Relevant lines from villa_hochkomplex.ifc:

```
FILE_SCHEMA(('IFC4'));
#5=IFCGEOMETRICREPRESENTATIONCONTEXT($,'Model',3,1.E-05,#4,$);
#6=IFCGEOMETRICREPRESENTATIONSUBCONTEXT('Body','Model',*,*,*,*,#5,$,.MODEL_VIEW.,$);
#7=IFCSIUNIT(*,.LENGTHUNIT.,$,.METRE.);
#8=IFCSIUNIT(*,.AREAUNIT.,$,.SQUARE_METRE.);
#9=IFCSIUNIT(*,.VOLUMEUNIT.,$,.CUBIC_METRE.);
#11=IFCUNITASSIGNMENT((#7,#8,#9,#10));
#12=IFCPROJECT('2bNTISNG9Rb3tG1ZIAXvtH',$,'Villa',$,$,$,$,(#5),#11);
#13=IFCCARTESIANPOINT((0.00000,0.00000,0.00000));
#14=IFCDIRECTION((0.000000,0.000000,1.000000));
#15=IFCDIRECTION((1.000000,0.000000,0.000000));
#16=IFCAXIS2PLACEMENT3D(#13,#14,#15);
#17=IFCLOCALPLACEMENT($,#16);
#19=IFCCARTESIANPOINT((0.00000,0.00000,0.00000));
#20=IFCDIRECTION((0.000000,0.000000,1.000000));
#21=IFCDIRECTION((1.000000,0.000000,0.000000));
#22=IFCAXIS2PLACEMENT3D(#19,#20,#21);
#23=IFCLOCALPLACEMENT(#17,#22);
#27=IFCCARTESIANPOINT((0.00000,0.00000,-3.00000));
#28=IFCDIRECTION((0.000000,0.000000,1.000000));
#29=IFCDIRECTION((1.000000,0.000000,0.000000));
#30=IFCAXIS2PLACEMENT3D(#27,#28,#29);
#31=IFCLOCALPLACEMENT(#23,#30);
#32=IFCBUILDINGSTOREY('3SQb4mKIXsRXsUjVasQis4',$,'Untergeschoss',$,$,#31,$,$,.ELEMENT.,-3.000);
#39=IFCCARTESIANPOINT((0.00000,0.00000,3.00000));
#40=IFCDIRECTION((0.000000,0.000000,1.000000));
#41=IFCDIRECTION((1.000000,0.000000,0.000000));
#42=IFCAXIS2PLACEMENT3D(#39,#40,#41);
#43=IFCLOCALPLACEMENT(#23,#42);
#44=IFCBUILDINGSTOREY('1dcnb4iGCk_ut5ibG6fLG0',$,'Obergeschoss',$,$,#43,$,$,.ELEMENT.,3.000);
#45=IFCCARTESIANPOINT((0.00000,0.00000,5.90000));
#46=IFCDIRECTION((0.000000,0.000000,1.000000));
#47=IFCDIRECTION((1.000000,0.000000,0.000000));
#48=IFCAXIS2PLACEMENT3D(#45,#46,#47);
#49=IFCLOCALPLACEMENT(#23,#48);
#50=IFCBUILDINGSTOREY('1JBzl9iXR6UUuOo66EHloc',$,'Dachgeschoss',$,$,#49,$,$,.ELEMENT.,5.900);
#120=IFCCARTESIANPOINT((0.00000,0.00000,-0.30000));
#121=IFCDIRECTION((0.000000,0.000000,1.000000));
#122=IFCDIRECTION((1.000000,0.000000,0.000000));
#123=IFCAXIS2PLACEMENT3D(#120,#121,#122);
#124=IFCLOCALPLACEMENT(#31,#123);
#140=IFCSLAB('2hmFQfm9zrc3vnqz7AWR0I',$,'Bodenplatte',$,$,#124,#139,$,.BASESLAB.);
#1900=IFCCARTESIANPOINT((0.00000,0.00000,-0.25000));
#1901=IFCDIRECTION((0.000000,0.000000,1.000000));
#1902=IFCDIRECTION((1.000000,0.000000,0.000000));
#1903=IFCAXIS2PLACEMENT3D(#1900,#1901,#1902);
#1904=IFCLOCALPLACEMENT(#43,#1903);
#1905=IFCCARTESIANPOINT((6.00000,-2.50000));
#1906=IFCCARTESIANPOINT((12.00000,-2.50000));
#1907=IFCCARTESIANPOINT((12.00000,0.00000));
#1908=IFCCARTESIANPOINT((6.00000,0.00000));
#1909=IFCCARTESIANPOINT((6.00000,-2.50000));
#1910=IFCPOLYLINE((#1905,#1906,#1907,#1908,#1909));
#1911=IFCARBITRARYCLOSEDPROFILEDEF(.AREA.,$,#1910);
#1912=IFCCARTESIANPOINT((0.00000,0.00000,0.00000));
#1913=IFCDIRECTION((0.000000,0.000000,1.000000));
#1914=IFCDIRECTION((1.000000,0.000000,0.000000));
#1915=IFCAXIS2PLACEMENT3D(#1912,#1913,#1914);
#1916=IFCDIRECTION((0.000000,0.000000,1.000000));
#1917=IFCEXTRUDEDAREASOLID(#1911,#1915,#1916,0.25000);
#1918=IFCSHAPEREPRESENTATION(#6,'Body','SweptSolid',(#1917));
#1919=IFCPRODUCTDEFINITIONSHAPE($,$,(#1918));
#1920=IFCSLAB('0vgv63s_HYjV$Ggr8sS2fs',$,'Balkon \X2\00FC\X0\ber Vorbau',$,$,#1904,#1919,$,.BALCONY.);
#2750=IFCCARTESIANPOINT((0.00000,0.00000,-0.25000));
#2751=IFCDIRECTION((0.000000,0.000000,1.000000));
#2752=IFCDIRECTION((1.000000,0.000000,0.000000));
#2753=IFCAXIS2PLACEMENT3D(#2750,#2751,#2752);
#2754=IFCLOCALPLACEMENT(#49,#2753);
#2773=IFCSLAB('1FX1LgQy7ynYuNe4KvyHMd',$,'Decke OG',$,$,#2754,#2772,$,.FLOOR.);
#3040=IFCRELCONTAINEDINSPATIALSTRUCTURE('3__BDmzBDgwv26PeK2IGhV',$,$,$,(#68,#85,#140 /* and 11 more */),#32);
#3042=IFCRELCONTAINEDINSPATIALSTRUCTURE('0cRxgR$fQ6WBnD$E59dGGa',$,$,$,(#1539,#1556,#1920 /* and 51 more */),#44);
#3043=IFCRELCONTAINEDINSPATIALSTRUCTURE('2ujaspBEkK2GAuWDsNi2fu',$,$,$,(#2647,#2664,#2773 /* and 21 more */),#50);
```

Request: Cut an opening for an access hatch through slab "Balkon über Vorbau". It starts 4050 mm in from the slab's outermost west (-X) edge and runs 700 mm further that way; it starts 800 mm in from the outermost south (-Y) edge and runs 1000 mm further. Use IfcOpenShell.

```python
import numpy as np
import ifcopenshell
import ifcopenshell.api.feature
import ifcopenshell.api.geometry
import ifcopenshell.api.root
import ifcopenshell.geom
import ifcopenshell.util.placement
import ifcopenshell.util.representation
import ifcopenshell.util.shape
import ifcopenshell.util.unit

model = ifcopenshell.open("villa_hochkomplex.ifc")
unit_scale = ifcopenshell.util.unit.calculate_unit_scale(model)
settings = ifcopenshell.geom.settings()


def volume(element):
    """Net volume in cubic metres, openings subtracted."""
    shape = ifcopenshell.geom.create_shape(settings, element)
    return ifcopenshell.util.shape.get_volume(shape.geometry)


slab = model.by_guid("0vgv63s_HYjV$Ggr8sS2fs")
before = volume(slab)

# Extent in the slab's own axes, in metres. The edges named are its -X and -Y sides.
slab_shape = ifcopenshell.geom.create_shape(settings, slab)
vertices = ifcopenshell.util.shape.get_vertices(slab_shape.geometry)
x_min, y_min, bottom = vertices.min(axis=0)
top = vertices[:, 2].max()

opening = ifcopenshell.api.root.create_entity(model, ifc_class="IfcOpeningElement", name="Access hatch opening", predefined_type="OPENING")
context = ifcopenshell.util.representation.get_context(model, "Model", "Body", "MODEL_VIEW")
width, depth = 0.7, 1
outline = [(0.0, 0.0), (width, 0.0), (width, depth), (0.0, depth), (0.0, 0.0)]
# Overshoot both faces by 50 mm so the cut is clean.
shape = ifcopenshell.api.geometry.add_slab_representation(
    model, context=context, depth=top - bottom + 0.1, polyline=outline
)
ifcopenshell.api.geometry.assign_representation(model, product=opening, representation=shape)

matrix = ifcopenshell.util.placement.get_local_placement(slab.ObjectPlacement)
matrix[:, 3] = matrix @ np.append(np.array([x_min + 4.05, y_min + 0.8, bottom - 0.05]) / unit_scale, 1.0)
ifcopenshell.api.geometry.edit_object_placement(model, product=opening, matrix=matrix, is_si=False)
ifcopenshell.api.feature.add_feature(model, feature=opening, element=slab)

after = volume(slab)

print(f"slab volume {before:.3f} -> {after:.3f} m3")

model.write("villa_hochkomplex-out.ifc")
```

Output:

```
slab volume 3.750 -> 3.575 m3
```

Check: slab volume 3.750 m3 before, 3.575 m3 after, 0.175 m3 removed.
